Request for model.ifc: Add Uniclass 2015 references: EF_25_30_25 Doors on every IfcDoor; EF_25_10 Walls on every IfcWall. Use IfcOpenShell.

First a look at what the model holds.

```python
import ifcopenshell

model = ifcopenshell.open("model.ifc")
print(model.schema)
print("classifications:", [c.Name for c in model.by_type("IfcClassification")])
for ifc_class in ("IfcDoor", "IfcRoof", "IfcStair", "IfcWall", "IfcWindow"):
    print(ifc_class, len(model.by_type(ifc_class)))
```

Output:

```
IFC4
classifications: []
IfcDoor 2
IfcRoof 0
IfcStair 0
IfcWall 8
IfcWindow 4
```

```python
import ifcopenshell
import ifcopenshell.api.classification

model = ifcopenshell.open("model.ifc")

system = ifcopenshell.api.classification.add_classification(model, classification="Uniclass 2015")

codes = {
    "IfcDoor": ("EF_25_30_25", "Doors"),
    "IfcWall": ("EF_25_10", "Walls"),
}
for ifc_class, (code, name) in codes.items():
    products = model.by_type(ifc_class)
    ifcopenshell.api.classification.add_reference(
        model, products=products, classification=system, identification=code, name=name
    )
    print(code, len(products))

model.write("model_v2.ifc")
```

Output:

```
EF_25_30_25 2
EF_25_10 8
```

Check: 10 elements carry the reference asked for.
